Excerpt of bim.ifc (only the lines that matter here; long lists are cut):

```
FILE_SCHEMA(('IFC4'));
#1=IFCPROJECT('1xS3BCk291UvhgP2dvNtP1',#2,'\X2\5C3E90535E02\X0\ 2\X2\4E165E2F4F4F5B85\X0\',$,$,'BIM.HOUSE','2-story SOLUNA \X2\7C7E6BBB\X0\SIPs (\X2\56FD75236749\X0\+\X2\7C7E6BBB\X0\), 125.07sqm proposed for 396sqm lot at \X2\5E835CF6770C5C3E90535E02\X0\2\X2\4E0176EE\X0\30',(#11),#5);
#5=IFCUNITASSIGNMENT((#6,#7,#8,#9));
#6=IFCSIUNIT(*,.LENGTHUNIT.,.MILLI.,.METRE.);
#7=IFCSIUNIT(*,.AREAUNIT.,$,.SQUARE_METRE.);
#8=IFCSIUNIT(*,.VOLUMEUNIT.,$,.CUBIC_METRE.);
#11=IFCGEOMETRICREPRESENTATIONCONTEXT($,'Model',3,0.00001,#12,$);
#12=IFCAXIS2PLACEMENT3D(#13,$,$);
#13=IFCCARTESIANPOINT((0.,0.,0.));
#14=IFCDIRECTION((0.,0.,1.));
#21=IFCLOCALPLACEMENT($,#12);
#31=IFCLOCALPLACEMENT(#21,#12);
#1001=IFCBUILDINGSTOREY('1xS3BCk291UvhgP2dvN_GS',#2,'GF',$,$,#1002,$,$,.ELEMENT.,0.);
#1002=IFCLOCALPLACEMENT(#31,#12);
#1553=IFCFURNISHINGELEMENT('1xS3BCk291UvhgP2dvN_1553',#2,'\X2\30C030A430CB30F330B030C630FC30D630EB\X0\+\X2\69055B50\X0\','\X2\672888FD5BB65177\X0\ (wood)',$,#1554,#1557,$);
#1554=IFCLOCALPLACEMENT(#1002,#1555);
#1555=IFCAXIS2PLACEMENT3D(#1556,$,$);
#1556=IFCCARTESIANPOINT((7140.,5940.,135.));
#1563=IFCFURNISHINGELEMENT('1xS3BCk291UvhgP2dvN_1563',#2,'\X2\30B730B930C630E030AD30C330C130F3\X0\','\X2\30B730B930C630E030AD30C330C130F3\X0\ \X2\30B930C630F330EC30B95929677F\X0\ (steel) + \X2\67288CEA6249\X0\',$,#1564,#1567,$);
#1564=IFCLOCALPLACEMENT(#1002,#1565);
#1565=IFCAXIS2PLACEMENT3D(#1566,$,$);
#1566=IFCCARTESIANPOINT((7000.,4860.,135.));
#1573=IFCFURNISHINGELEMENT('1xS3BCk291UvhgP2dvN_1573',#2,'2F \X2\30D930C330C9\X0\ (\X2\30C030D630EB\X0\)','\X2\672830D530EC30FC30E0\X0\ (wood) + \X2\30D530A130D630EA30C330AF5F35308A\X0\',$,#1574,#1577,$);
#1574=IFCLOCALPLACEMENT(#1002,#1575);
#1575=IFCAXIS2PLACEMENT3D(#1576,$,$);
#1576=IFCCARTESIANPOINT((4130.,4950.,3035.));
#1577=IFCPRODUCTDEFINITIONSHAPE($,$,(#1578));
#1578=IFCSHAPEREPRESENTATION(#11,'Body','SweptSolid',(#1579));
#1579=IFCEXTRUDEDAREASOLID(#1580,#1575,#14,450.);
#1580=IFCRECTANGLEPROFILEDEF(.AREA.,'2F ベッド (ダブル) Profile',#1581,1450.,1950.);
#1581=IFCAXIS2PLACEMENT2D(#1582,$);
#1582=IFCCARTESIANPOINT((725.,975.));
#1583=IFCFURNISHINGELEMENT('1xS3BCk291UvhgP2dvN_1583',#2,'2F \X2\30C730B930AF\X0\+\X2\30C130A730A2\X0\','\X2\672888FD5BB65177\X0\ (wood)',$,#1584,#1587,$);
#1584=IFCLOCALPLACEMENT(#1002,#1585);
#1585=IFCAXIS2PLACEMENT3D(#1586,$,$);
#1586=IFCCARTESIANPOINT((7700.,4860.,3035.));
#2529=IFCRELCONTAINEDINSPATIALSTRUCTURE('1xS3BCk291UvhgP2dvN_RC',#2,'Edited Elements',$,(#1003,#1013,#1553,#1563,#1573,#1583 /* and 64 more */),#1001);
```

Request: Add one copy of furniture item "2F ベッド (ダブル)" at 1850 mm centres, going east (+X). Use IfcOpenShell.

```python
import numpy as np
import ifcopenshell
import ifcopenshell.api.geometry
import ifcopenshell.api.root
import ifcopenshell.util.element
import ifcopenshell.util.placement
import ifcopenshell.util.unit

model = ifcopenshell.open("bim.ifc")
unit_scale = ifcopenshell.util.unit.calculate_unit_scale(model)


def reuse_history(source, copy):
    """copy_class also copies each property set's owner history, people and application; keep the originals."""
    for rel in copy.IsDefinedBy:
        if rel.is_a("IfcRelDefinesByProperties") and (history := rel.RelatingPropertyDefinition.OwnerHistory):
            rel.RelatingPropertyDefinition.OwnerHistory = source.OwnerHistory
            ifcopenshell.util.element.remove_deep2(model, history)


source = model.by_id(1573)
base = ifcopenshell.util.placement.get_local_placement(source.ObjectPlacement)
step = np.array([1.0, 0.0, 0.0]) * 1.85 / unit_scale

for i in range(1, 2):
    copy = ifcopenshell.api.root.copy_class(model, product=source)
    copy.Representation = ifcopenshell.util.element.copy_deep(
        model, source.Representation, exclude=["IfcGeometricRepresentationContext", "IfcRepresentationMap"]
    )
    reuse_history(source, copy)
    matrix = base.copy()
    matrix[:3, 3] += i * step
    print("added at", matrix[:3, 3].round(3) + 0.0)
    ifcopenshell.api.geometry.edit_object_placement(model, product=copy, matrix=matrix, is_si=False)

model.write("bim_edited.ifc")
```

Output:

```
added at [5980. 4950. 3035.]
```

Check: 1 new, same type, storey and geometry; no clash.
